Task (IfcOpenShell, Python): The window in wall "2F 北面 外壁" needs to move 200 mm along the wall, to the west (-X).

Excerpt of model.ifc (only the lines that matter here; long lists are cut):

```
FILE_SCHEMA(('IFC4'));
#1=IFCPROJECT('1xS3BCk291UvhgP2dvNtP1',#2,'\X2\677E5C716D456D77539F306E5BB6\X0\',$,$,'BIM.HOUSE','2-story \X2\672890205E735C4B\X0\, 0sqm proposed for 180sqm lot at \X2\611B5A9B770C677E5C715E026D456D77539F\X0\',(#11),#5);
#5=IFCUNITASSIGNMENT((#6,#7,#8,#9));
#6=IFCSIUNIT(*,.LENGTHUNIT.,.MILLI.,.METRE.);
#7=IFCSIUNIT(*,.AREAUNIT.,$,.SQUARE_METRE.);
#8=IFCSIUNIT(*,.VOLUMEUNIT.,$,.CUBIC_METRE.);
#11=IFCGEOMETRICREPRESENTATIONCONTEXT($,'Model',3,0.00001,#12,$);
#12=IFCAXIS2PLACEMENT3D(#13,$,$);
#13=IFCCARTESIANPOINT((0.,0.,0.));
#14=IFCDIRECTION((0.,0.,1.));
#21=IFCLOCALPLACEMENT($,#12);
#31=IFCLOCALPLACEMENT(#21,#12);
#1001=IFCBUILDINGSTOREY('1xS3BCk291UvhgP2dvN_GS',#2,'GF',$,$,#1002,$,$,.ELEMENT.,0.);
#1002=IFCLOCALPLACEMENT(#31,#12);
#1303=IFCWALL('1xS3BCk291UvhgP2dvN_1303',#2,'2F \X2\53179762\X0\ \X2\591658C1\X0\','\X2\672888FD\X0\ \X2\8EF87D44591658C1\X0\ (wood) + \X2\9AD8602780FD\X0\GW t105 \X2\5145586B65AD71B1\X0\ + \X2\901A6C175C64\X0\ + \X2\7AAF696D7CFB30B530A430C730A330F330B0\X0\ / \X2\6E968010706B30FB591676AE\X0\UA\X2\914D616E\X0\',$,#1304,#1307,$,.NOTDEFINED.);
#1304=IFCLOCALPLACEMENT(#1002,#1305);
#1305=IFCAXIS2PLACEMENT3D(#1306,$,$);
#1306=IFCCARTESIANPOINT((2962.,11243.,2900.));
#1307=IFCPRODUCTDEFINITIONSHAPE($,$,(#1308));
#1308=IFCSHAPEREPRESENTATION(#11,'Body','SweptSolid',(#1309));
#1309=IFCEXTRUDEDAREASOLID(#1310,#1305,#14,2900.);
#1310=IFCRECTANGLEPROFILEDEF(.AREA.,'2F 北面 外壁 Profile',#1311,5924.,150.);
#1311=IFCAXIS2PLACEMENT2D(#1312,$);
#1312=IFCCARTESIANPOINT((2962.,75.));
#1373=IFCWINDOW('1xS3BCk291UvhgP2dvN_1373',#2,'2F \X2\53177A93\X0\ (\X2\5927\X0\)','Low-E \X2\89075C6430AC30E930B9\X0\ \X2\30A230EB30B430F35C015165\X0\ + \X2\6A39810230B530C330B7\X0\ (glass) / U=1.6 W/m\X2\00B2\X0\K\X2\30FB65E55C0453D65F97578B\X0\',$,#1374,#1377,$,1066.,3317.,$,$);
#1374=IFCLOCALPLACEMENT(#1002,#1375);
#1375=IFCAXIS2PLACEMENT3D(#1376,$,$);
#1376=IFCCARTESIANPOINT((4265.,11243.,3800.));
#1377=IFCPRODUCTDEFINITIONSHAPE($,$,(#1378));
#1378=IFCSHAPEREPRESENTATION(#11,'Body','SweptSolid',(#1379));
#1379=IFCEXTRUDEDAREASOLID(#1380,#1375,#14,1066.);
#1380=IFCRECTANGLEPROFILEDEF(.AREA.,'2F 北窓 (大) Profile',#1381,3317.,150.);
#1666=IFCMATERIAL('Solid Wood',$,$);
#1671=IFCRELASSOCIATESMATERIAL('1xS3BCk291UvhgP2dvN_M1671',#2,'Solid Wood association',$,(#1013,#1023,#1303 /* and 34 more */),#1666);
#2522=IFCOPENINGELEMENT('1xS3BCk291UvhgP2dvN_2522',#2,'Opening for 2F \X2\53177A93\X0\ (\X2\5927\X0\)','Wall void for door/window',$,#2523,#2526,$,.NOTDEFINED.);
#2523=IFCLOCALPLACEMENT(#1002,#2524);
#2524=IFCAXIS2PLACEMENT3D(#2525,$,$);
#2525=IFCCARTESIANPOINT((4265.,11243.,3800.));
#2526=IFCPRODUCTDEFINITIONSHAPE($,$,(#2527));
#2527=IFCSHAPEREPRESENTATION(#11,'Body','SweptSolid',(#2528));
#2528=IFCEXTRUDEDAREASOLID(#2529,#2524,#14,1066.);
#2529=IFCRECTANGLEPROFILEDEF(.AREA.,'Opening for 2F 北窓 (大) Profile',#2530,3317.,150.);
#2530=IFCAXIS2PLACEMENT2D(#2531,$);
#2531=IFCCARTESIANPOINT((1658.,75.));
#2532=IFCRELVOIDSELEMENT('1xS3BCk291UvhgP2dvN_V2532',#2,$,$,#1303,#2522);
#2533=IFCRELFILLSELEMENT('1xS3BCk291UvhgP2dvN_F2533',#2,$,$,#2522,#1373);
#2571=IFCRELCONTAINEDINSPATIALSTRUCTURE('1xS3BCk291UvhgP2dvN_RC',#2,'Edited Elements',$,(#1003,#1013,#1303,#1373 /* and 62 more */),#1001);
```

```python
import ifcopenshell
import ifcopenshell.api.geometry
import ifcopenshell.util.placement
import ifcopenshell.util.unit

model = ifcopenshell.open("model.ifc")
unit_scale = ifcopenshell.util.unit.calculate_unit_scale(model)

window = model.by_id(1373)
opening = window.FillsVoids[0].RelatingOpeningElement
wall = opening.VoidsElements[0].RelatingBuildingElement

wall_matrix = ifcopenshell.util.placement.get_local_placement(wall.ObjectPlacement)
shift = wall_matrix[:3, 0] * -0.2 / unit_scale
before = ifcopenshell.util.placement.get_local_placement(window.ObjectPlacement)[:3, 3].copy()

# The window is not placed relative to its opening, so move both.
for product in (opening, window):
    matrix = ifcopenshell.util.placement.get_local_placement(product.ObjectPlacement)
    matrix[:3, 3] += shift
    ifcopenshell.api.geometry.edit_object_placement(model, product=product, matrix=matrix, is_si=False)

after = ifcopenshell.util.placement.get_local_placement(window.ObjectPlacement)[:3, 3]
print("window moved by", (after - before).round(3) + 0.0)

model.write("model_rev.ifc")
```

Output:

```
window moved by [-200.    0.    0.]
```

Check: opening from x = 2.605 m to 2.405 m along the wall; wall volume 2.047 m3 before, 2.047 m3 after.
